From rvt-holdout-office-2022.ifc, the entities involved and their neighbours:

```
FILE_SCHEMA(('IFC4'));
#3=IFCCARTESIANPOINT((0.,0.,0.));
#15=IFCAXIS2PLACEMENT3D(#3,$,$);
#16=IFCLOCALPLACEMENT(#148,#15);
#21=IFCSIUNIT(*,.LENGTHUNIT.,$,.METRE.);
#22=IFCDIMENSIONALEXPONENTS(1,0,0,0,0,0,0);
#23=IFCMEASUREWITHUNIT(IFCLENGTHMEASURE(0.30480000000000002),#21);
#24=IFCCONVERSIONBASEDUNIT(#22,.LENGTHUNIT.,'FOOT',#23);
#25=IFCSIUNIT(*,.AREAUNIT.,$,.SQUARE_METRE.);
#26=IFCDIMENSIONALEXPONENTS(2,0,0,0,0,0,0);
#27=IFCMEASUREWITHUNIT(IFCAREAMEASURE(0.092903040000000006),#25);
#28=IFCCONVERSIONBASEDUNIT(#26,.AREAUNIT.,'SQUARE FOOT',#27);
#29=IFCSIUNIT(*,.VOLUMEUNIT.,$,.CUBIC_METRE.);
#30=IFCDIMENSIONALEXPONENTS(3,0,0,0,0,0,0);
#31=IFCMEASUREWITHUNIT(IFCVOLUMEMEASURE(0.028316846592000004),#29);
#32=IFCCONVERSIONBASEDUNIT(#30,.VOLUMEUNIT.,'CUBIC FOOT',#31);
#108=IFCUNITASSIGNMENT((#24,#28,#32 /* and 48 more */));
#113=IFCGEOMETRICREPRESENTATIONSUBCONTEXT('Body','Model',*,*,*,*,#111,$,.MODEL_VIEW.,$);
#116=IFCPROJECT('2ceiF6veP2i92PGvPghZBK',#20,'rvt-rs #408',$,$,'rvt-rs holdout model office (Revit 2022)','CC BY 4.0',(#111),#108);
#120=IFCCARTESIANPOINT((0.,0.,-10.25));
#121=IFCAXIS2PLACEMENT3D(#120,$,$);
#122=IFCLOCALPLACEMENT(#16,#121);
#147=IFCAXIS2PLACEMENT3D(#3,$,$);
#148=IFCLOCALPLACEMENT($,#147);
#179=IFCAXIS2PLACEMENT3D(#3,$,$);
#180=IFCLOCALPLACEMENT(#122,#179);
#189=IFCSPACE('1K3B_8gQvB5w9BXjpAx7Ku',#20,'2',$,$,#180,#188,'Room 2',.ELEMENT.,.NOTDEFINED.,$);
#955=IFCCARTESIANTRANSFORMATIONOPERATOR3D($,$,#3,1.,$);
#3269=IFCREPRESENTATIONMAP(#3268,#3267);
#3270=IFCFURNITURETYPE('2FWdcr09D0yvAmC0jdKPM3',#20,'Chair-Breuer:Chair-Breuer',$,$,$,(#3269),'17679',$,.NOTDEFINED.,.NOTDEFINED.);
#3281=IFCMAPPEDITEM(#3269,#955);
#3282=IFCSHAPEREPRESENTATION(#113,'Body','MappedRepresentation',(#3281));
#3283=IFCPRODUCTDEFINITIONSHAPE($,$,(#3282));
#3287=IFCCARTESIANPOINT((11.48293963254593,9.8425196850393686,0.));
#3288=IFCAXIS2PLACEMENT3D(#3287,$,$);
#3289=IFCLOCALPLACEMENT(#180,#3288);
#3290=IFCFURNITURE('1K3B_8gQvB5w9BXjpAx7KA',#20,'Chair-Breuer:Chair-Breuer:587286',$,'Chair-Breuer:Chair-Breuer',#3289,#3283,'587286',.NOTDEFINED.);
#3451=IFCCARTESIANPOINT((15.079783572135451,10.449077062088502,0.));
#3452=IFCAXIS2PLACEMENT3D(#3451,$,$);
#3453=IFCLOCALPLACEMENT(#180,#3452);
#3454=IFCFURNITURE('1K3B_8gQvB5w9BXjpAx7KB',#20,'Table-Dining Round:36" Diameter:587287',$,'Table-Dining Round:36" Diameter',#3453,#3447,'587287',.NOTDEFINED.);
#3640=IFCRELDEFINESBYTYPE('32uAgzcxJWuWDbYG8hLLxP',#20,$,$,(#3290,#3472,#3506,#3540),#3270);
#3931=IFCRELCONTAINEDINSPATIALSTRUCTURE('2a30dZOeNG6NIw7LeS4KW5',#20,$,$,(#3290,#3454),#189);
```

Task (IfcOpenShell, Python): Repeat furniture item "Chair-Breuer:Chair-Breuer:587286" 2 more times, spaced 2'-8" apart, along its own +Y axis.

```python
import ifcopenshell
import ifcopenshell.api.geometry
import ifcopenshell.api.root
import ifcopenshell.util.element
import ifcopenshell.util.placement
import ifcopenshell.util.unit

model = ifcopenshell.open("rvt-holdout-office-2022.ifc")
unit_scale = ifcopenshell.util.unit.calculate_unit_scale(model)


def reuse_history(source, copy):
    """copy_class also copies each property set's owner history, people and application; keep the originals."""
    for rel in copy.IsDefinedBy:
        if rel.is_a("IfcRelDefinesByProperties") and (history := rel.RelatingPropertyDefinition.OwnerHistory):
            rel.RelatingPropertyDefinition.OwnerHistory = source.OwnerHistory
            ifcopenshell.util.element.remove_deep2(model, history)


source = model.by_guid("1K3B_8gQvB5w9BXjpAx7KA")
base = ifcopenshell.util.placement.get_local_placement(source.ObjectPlacement)
step = base[:3, 1] * 32 * 0.0254 / unit_scale

for i in range(1, 3):
    copy = ifcopenshell.api.root.copy_class(model, product=source)
    copy.Representation = ifcopenshell.util.element.copy_deep(
        model, source.Representation, exclude=["IfcGeometricRepresentationContext", "IfcRepresentationMap"]
    )
    copy.Name = "Chair-Breuer:Chair-Breuer"
    copy.Tag = None
    reuse_history(source, copy)
    matrix = base.copy()
    matrix[:3, 3] += i * step
    print("added at", matrix[:3, 3].round(3) + 0.0)
    ifcopenshell.api.geometry.edit_object_placement(model, product=copy, matrix=matrix, is_si=False)

model.write("rvt-holdout-office-2022-out.ifc")
```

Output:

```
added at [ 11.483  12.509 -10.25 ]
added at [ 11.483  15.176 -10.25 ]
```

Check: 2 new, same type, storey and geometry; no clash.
